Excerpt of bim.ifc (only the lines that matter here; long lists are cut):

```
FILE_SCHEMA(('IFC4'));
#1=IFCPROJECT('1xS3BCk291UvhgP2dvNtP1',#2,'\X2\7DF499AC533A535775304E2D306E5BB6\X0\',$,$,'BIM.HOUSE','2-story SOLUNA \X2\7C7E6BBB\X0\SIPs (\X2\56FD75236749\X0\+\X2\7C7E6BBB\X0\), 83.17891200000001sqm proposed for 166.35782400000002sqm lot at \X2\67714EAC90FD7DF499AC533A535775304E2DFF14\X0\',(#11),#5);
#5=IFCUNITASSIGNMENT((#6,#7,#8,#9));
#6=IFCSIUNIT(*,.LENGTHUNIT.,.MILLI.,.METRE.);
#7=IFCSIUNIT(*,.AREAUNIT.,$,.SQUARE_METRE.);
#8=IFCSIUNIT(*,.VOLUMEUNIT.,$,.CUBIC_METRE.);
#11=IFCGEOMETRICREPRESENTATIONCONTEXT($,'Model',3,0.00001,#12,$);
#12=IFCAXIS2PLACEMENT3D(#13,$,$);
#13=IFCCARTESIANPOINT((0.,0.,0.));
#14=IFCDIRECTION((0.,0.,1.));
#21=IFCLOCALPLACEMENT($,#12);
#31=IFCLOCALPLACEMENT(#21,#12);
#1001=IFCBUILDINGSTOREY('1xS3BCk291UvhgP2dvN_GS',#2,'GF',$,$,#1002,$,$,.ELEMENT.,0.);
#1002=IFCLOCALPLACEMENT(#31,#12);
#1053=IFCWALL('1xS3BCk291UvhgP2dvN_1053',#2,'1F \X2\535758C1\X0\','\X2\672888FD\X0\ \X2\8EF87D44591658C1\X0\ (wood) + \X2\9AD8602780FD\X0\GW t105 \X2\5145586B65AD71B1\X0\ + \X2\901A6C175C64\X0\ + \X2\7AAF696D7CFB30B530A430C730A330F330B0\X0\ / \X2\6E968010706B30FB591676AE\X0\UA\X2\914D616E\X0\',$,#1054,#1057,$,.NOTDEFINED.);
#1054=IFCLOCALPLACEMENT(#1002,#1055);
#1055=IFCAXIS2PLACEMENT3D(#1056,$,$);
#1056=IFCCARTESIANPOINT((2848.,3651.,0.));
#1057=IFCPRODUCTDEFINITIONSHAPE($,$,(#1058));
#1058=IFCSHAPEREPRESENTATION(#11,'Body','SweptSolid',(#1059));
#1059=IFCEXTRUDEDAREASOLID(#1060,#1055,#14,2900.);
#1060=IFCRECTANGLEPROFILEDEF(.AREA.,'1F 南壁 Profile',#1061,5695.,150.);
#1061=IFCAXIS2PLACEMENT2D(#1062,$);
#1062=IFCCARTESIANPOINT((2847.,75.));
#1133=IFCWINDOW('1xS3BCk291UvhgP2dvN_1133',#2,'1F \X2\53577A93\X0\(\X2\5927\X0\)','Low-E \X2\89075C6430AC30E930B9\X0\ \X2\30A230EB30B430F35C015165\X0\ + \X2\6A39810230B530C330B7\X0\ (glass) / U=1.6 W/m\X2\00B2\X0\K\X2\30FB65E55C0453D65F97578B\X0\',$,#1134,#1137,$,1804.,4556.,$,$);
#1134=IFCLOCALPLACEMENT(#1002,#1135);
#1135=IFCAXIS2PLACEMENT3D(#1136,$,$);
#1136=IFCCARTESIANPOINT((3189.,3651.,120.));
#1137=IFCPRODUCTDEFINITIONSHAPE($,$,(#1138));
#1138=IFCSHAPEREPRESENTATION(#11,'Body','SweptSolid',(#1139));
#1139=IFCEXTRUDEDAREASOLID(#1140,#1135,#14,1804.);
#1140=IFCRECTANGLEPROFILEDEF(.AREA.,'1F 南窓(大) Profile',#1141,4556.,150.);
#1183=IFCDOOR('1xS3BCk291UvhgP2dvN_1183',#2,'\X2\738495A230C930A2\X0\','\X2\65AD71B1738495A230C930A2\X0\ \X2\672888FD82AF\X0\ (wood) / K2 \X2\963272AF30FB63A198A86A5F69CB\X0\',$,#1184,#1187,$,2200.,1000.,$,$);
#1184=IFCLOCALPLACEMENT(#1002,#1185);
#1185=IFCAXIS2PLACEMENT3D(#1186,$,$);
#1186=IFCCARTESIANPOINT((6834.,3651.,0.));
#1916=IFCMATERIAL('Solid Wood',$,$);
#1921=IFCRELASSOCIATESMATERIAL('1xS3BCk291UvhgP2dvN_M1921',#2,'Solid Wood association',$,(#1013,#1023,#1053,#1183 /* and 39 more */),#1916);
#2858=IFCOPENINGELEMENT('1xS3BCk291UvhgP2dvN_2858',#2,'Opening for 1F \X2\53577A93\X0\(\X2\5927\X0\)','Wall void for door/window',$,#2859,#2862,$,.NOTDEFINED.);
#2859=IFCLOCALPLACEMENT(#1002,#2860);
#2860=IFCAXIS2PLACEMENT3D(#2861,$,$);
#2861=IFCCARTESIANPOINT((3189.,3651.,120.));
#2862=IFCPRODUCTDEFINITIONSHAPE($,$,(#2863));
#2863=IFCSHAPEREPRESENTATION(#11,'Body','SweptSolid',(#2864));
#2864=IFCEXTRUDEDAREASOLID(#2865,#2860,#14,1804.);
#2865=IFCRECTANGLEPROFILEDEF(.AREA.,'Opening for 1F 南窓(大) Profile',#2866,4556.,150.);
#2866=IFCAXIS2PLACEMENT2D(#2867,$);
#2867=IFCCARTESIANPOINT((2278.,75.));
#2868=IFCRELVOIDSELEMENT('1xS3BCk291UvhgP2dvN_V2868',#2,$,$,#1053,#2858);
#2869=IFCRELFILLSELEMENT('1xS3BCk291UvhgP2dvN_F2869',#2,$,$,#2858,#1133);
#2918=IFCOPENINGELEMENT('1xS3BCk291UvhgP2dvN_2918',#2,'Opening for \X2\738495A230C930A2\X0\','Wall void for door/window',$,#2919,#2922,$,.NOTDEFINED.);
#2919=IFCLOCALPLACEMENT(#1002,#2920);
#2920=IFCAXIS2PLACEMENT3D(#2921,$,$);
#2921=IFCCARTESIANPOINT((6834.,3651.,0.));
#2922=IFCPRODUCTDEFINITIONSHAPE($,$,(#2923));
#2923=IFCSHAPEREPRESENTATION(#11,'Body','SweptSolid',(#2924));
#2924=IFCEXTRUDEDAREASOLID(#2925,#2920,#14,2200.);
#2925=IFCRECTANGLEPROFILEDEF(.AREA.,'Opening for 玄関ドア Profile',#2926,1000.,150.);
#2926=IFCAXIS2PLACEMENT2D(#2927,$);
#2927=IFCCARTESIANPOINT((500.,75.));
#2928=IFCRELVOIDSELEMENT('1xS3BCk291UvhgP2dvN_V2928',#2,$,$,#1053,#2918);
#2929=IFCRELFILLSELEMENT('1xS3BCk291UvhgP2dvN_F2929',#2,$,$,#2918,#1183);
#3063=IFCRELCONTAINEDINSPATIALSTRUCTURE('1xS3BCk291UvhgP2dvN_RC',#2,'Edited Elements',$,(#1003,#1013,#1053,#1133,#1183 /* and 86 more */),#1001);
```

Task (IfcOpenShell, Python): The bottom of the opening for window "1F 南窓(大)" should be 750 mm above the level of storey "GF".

```python
import numpy as np
import ifcopenshell
import ifcopenshell.api.geometry
import ifcopenshell.geom
import ifcopenshell.util.element
import ifcopenshell.util.placement
import ifcopenshell.util.shape
import ifcopenshell.util.unit

model = ifcopenshell.open("bim.ifc")
unit_scale = ifcopenshell.util.unit.calculate_unit_scale(model)

window = model.by_guid("1xS3BCk291UvhgP2dvN_1133")
opening = window.FillsVoids[0].RelatingOpeningElement
storey = ifcopenshell.util.element.get_container(window, ifc_class="IfcBuildingStorey")
level = ifcopenshell.util.placement.get_local_placement(storey.ObjectPlacement)[2, 3]

# The opening's origin need not be at the sill, so measure its lowest point.
shape = ifcopenshell.geom.create_shape(ifcopenshell.geom.settings(), opening)
bottom = ifcopenshell.util.shape.get_shape_bottom_elevation(shape, shape.geometry) / unit_scale
dz = level + 0.75 / unit_scale - bottom

shift = np.array([0.0, 0.0, dz])
# The window is not placed relative to its opening, so move both.
for product in (opening, window):
    matrix = ifcopenshell.util.placement.get_local_placement(product.ObjectPlacement)
    matrix[:3, 3] += shift
    ifcopenshell.api.geometry.edit_object_placement(model, product=product, matrix=matrix, is_si=False)

print(f"moved by {dz * unit_scale:+.3f} m")

model.write("bim_v2.ifc")
```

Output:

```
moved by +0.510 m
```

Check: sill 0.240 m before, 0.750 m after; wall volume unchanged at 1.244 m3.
